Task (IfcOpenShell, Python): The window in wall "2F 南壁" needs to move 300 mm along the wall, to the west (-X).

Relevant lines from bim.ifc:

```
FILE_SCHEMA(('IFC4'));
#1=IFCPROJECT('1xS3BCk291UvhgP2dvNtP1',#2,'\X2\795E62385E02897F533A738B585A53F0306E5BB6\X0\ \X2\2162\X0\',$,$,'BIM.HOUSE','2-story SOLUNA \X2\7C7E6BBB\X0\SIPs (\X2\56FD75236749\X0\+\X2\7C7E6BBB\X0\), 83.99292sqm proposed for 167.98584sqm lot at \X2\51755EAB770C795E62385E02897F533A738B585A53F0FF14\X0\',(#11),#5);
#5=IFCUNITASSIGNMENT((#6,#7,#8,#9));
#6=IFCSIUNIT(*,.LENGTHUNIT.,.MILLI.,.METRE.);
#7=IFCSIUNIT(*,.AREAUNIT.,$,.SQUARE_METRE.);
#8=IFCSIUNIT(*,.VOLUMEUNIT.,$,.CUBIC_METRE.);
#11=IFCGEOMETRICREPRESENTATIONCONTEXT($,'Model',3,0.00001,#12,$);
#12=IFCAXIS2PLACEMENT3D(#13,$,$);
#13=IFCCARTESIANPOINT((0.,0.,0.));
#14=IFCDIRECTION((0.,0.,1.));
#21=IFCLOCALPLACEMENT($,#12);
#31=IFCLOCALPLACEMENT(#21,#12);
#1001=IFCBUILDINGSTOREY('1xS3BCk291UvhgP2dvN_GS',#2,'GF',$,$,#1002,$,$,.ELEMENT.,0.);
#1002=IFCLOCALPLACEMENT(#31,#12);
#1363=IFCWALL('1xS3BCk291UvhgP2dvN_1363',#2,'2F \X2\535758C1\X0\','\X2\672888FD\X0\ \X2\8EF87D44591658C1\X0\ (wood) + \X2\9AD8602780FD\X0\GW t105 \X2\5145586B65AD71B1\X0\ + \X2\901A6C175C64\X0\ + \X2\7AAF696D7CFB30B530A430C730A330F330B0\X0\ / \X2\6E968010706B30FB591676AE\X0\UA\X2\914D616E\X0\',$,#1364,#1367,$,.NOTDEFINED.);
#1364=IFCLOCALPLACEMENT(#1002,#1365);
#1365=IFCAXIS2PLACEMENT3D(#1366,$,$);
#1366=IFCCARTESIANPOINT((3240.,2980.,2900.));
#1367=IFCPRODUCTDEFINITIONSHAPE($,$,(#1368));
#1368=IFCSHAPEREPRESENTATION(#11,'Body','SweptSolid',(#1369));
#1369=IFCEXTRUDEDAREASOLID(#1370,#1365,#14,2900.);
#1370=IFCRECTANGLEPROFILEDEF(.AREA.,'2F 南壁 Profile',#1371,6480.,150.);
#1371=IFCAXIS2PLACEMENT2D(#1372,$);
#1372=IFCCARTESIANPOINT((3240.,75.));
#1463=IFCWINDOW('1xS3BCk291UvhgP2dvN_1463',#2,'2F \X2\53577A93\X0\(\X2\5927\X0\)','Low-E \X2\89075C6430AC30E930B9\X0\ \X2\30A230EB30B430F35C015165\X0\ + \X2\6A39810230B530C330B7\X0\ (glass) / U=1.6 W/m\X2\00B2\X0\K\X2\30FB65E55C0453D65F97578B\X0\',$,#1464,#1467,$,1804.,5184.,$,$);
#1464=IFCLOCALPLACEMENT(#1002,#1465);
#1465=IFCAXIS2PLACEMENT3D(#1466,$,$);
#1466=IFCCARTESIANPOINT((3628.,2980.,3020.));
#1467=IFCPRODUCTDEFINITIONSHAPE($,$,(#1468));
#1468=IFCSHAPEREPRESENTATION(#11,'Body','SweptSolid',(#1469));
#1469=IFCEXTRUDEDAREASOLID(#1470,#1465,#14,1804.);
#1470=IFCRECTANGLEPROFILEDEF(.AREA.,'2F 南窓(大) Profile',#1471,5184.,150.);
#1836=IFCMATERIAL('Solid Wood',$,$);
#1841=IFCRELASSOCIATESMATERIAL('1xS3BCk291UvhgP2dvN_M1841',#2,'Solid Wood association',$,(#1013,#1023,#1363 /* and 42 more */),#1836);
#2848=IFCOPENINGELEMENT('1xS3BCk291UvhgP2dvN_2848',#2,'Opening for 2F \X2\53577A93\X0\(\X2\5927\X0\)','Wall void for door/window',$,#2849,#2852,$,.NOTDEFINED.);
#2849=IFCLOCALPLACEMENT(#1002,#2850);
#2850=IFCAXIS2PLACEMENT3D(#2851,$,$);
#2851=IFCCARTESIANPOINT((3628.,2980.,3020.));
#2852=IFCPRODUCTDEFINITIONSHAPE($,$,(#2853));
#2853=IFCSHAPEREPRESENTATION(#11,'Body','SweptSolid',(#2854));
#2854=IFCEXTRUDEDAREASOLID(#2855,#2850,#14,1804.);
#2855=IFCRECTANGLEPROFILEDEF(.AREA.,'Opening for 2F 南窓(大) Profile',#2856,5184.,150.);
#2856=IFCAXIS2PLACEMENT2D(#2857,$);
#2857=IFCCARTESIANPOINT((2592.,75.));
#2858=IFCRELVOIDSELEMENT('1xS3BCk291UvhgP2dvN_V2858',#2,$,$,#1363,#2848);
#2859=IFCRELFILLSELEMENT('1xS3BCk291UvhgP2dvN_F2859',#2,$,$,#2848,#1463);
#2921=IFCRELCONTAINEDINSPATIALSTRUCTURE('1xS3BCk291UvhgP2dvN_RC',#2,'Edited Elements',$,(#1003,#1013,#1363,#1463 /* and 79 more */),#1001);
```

```python
import ifcopenshell
import ifcopenshell.api.geometry
import ifcopenshell.util.placement
import ifcopenshell.util.unit

model = ifcopenshell.open("bim.ifc")
unit_scale = ifcopenshell.util.unit.calculate_unit_scale(model)

window = model.by_id(1463)
opening = window.FillsVoids[0].RelatingOpeningElement
wall = opening.VoidsElements[0].RelatingBuildingElement

wall_matrix = ifcopenshell.util.placement.get_local_placement(wall.ObjectPlacement)
shift = wall_matrix[:3, 0] * -0.3 / unit_scale
before = ifcopenshell.util.placement.get_local_placement(window.ObjectPlacement)[:3, 3].copy()

# The window is not placed relative to its opening, so move both.
for product in (opening, window):
    matrix = ifcopenshell.util.placement.get_local_placement(product.ObjectPlacement)
    matrix[:3, 3] += shift
    ifcopenshell.api.geometry.edit_object_placement(model, product=product, matrix=matrix, is_si=False)

after = ifcopenshell.util.placement.get_local_placement(window.ObjectPlacement)[:3, 3]
print("window moved by", (after - before).round(3) + 0.0)

model.write("bim_edited.ifc")
```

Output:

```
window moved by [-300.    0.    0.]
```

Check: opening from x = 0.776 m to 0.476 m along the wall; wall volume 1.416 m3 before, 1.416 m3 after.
